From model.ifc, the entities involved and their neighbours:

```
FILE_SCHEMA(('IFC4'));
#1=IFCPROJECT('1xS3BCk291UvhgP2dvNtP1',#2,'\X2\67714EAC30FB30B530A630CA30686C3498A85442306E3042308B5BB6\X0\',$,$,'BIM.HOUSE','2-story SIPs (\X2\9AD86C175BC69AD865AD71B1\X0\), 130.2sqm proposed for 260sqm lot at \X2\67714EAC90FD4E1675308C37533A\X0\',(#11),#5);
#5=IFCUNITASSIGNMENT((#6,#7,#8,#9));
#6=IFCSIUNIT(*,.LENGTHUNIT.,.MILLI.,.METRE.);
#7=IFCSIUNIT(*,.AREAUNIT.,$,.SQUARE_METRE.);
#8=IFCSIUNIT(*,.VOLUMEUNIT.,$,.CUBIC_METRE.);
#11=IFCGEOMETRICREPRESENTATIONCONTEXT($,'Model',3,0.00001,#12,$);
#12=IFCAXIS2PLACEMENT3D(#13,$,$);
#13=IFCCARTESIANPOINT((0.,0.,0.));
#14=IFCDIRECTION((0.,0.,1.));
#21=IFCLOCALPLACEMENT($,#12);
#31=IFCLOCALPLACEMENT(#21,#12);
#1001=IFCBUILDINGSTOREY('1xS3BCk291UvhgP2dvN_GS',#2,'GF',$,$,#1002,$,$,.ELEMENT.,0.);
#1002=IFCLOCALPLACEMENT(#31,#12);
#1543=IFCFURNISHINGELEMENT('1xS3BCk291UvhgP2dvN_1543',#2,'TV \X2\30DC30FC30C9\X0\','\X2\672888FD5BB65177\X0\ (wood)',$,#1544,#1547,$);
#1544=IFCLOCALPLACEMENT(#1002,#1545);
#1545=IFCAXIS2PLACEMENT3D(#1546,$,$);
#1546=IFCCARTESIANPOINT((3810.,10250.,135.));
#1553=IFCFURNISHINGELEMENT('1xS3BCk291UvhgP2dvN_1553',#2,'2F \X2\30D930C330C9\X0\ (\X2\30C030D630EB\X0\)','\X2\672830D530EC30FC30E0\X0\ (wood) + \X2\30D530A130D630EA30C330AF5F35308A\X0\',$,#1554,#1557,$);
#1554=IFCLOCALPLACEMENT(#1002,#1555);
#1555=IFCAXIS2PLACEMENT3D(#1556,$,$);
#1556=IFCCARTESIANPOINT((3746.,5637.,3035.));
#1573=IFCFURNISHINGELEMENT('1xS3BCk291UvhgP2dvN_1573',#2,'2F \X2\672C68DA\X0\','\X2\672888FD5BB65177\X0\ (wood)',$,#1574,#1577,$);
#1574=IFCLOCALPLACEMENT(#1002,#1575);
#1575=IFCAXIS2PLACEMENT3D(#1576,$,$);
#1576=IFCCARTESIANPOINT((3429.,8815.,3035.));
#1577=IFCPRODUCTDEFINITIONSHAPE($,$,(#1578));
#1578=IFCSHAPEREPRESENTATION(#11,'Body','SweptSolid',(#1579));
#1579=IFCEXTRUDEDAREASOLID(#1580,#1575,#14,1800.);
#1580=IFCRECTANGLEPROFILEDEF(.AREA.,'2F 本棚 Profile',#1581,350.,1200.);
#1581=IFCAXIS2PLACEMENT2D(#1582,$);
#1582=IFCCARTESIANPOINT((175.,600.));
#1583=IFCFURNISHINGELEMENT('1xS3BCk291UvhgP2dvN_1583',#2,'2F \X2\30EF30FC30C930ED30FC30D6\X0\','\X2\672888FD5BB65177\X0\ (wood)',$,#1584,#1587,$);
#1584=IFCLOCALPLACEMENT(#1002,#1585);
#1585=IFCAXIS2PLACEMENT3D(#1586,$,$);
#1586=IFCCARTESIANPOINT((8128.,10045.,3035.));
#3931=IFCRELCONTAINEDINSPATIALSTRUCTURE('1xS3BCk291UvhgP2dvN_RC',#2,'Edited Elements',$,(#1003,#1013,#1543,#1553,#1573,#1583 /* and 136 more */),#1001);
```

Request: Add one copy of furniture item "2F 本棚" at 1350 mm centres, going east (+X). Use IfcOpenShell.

```python
import numpy as np
import ifcopenshell
import ifcopenshell.api.geometry
import ifcopenshell.api.root
import ifcopenshell.util.element
import ifcopenshell.util.placement
import ifcopenshell.util.unit

model = ifcopenshell.open("model.ifc")
unit_scale = ifcopenshell.util.unit.calculate_unit_scale(model)


def reuse_history(source, copy):
    """copy_class also copies each property set's owner history, people and application; keep the originals."""
    for rel in copy.IsDefinedBy:
        if rel.is_a("IfcRelDefinesByProperties") and (history := rel.RelatingPropertyDefinition.OwnerHistory):
            rel.RelatingPropertyDefinition.OwnerHistory = source.OwnerHistory
            ifcopenshell.util.element.remove_deep2(model, history)


source = model.by_id(1573)
base = ifcopenshell.util.placement.get_local_placement(source.ObjectPlacement)
step = np.array([1.0, 0.0, 0.0]) * 1.35 / unit_scale

for i in range(1, 2):
    copy = ifcopenshell.api.root.copy_class(model, product=source)
    copy.Representation = ifcopenshell.util.element.copy_deep(
        model, source.Representation, exclude=["IfcGeometricRepresentationContext", "IfcRepresentationMap"]
    )
    reuse_history(source, copy)
    matrix = base.copy()
    matrix[:3, 3] += i * step
    print("added at", matrix[:3, 3].round(3) + 0.0)
    ifcopenshell.api.geometry.edit_object_placement(model, product=copy, matrix=matrix, is_si=False)

model.write("model-out.ifc")
```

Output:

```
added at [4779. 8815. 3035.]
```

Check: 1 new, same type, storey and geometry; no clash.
